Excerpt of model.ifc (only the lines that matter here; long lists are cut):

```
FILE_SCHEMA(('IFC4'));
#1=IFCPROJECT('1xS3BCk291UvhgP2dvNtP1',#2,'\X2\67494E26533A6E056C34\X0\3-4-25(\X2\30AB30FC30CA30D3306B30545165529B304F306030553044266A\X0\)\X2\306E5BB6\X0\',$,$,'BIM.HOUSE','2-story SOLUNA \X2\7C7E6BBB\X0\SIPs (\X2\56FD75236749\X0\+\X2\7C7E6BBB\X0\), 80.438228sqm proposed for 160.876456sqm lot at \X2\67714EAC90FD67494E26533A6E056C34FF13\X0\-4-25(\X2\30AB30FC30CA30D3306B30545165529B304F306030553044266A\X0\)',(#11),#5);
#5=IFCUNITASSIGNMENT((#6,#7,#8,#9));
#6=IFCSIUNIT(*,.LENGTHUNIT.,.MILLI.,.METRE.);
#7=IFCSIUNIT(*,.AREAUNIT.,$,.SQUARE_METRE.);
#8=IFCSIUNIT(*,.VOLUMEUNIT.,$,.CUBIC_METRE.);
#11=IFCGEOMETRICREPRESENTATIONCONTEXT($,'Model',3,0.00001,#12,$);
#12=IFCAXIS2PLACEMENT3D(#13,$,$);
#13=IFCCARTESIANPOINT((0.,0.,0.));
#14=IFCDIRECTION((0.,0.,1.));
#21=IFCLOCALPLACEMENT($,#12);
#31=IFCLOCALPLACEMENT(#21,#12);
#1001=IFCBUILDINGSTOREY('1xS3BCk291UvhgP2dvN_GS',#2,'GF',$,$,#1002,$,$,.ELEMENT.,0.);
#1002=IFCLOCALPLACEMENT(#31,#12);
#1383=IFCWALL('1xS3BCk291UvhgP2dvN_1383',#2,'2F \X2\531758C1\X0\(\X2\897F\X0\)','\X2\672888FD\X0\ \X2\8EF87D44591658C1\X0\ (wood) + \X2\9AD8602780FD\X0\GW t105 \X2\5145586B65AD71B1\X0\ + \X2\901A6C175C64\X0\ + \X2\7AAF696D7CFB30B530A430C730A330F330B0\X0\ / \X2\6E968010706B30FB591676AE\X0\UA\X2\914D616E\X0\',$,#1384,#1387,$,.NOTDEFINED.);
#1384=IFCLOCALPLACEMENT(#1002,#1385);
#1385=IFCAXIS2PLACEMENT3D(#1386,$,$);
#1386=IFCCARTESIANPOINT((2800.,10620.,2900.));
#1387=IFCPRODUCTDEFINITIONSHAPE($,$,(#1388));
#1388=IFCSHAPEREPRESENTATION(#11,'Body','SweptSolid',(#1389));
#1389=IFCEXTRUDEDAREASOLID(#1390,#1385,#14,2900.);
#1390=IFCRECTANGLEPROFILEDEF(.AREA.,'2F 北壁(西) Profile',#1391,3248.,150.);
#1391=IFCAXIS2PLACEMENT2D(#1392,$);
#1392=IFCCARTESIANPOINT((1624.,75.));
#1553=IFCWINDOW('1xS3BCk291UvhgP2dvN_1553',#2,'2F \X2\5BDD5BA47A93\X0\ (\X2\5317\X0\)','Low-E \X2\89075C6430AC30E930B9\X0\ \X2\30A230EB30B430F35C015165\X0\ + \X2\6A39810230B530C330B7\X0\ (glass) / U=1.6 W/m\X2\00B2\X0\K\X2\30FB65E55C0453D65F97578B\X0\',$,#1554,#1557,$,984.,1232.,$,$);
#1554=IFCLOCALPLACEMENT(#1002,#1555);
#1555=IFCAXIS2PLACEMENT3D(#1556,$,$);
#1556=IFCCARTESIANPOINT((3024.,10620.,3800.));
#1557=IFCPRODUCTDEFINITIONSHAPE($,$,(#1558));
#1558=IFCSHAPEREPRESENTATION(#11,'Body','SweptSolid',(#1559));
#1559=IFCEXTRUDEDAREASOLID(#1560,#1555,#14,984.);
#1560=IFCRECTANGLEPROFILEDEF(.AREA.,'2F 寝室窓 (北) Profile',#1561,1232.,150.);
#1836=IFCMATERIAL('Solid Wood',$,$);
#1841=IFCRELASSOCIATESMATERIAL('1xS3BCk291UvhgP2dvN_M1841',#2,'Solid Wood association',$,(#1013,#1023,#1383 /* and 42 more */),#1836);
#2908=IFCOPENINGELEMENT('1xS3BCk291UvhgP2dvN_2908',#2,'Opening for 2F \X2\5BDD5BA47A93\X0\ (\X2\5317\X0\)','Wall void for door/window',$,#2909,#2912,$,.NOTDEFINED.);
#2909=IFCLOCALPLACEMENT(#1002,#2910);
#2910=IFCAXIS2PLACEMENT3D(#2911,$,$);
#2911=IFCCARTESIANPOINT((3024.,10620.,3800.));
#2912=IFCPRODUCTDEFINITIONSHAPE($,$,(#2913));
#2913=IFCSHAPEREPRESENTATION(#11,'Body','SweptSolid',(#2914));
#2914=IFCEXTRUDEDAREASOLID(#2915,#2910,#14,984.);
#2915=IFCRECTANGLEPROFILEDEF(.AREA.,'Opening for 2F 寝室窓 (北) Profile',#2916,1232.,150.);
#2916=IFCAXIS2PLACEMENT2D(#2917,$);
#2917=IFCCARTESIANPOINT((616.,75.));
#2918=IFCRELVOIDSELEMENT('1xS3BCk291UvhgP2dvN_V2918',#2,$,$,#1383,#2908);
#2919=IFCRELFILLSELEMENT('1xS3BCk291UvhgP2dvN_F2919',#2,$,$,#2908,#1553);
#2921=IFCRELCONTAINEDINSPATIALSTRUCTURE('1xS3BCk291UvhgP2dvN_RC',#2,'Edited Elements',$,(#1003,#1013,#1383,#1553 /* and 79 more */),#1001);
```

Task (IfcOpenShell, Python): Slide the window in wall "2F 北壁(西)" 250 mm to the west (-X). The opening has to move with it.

```python
import ifcopenshell
import ifcopenshell.api.geometry
import ifcopenshell.util.placement

model = ifcopenshell.open("model.ifc")

window = model.by_id(1553)
opening = window.FillsVoids[0].RelatingOpeningElement
wall = opening.VoidsElements[0].RelatingBuildingElement

wall_matrix = ifcopenshell.util.placement.get_local_placement(wall.ObjectPlacement)
shift = wall_matrix[:3, 0] * -250.0
before = ifcopenshell.util.placement.get_local_placement(window.ObjectPlacement)[:3, 3].copy()

# The window is not placed relative to its opening, so move both.
for product in (opening, window):
    matrix = ifcopenshell.util.placement.get_local_placement(product.ObjectPlacement)
    matrix[:3, 3] += shift
    ifcopenshell.api.geometry.edit_object_placement(model, product=product, matrix=matrix, is_si=False)

after = ifcopenshell.util.placement.get_local_placement(window.ObjectPlacement)[:3, 3]
print("window moved by", (after - before).round(3) + 0.0)

model.write("model_updated.ifc")
```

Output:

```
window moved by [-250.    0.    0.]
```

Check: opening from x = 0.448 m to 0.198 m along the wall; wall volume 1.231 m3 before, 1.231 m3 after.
